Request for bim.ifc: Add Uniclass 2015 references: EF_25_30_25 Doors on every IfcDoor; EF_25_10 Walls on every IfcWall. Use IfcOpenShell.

First a look at what the model holds.

```python
import ifcopenshell

model = ifcopenshell.open("bim.ifc")
print(model.schema)
print("classifications:", [c.Name for c in model.by_type("IfcClassification")])
for ifc_class in ("IfcDoor", "IfcRoof", "IfcStair", "IfcWall", "IfcWindow"):
    print(ifc_class, len(model.by_type(ifc_class)))
```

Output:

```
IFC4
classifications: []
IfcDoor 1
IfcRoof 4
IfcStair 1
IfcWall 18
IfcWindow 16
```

```python
import ifcopenshell
import ifcopenshell.api.classification

model = ifcopenshell.open("bim.ifc")

system = ifcopenshell.api.classification.add_classification(model, classification="Uniclass 2015")

codes = {
    "IfcDoor": ("EF_25_30_25", "Doors"),
    "IfcWall": ("EF_25_10", "Walls"),
}
for ifc_class, (code, name) in codes.items():
    products = model.by_type(ifc_class)
    ifcopenshell.api.classification.add_reference(
        model, products=products, classification=system, identification=code, name=name
    )
    print(code, len(products))

model.write("bim_v2.ifc")
```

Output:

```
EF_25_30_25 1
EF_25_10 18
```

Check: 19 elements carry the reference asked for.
